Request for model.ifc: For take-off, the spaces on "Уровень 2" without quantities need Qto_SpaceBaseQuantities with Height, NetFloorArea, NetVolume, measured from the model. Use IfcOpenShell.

First a look at what the model holds.

```python
import ifcopenshell
import ifcopenshell.util.element
import ifcopenshell.util.unit

model = ifcopenshell.open("model.ifc")
print(model.schema)
for unit_type in ("LENGTHUNIT", "AREAUNIT", "VOLUMEUNIT"):
    print(unit_type, ifcopenshell.util.unit.calculate_unit_scale(model, unit_type))
storey = next(s for s in model.by_type("IfcBuildingStorey") if s.Name == "Уровень 2")
spaces = [e for e in ifcopenshell.util.element.get_decomposition(storey) if e.is_a("IfcSpace")]
for e in sorted(spaces, key=lambda e: e.id()):
    print(e.id(), e.is_a(), e.Name, list(ifcopenshell.util.element.get_psets(e, qtos_only=True)), sep=" | ")
```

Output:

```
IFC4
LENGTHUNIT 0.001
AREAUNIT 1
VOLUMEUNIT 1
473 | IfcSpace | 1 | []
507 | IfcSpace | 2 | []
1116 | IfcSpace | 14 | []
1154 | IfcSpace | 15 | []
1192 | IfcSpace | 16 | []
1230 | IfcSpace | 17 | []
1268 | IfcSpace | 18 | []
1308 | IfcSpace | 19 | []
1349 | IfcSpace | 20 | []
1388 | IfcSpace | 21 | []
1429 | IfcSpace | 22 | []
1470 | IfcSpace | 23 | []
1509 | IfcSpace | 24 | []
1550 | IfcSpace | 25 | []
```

```python
import ifcopenshell
import ifcopenshell.api.pset
import ifcopenshell.geom
import ifcopenshell.util.element
import ifcopenshell.util.shape
import ifcopenshell.util.unit

model = ifcopenshell.open("model.ifc")
unit_scale = ifcopenshell.util.unit.calculate_unit_scale(model)
area_scale = ifcopenshell.util.unit.calculate_unit_scale(model, "AREAUNIT")
volume_scale = ifcopenshell.util.unit.calculate_unit_scale(model, "VOLUMEUNIT")
settings = ifcopenshell.geom.settings()

storey = next(s for s in model.by_type("IfcBuildingStorey") if s.Name == "Уровень 2")
spaces = [e for e in ifcopenshell.util.element.get_decomposition(storey) if e.is_a("IfcSpace")]

for e in sorted(spaces, key=lambda e: e.id()):
    if ifcopenshell.util.element.get_psets(e, qtos_only=True, should_inherit=False):
        continue
    # Geometry comes back in metres, in the element's own axes.
    shape = ifcopenshell.geom.create_shape(settings, e)
    values = {
        "Height": ifcopenshell.util.shape.get_z(shape.geometry) / unit_scale,
        "NetFloorArea": ifcopenshell.util.shape.get_footprint_area(shape.geometry) / area_scale,
        "NetVolume": ifcopenshell.util.shape.get_volume(shape.geometry) / volume_scale,
    }
    qto = ifcopenshell.api.pset.add_qto(model, product=e, name="Qto_SpaceBaseQuantities")
    ifcopenshell.api.pset.edit_qto(model, qto=qto, properties=values)
    print(e.id(), {k: round(v, 3) for k, v in values.items()})

model.write("model_rev.ifc")
```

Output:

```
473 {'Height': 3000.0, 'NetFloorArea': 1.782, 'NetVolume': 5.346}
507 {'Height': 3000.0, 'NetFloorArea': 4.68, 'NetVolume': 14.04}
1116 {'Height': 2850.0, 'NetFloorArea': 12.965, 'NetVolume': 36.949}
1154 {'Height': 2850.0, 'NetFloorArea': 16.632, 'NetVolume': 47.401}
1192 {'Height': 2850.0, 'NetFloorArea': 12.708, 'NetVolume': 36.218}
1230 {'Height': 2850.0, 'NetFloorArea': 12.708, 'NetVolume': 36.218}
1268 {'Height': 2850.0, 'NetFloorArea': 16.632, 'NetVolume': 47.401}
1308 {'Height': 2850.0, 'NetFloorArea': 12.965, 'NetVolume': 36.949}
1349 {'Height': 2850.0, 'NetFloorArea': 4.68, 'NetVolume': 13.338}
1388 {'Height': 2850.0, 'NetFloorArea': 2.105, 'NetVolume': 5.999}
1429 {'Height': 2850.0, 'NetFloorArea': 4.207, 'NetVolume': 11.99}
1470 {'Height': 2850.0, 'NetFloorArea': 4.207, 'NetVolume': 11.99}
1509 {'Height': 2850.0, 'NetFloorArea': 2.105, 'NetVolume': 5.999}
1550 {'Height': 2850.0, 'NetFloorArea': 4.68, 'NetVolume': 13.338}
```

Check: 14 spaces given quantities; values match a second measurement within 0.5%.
